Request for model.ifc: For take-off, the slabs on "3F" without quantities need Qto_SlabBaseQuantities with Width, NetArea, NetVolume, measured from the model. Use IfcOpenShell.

First a look at what the model holds.

```python
import ifcopenshell
import ifcopenshell.util.element
import ifcopenshell.util.unit

model = ifcopenshell.open("model.ifc")
print(model.schema)
for unit_type in ("LENGTHUNIT", "AREAUNIT", "VOLUMEUNIT"):
    print(unit_type, ifcopenshell.util.unit.calculate_unit_scale(model, unit_type))
storey = next(s for s in model.by_type("IfcBuildingStorey") if s.Name == "3F")
slabs = [e for e in ifcopenshell.util.element.get_decomposition(storey) if e.is_a("IfcSlab")]
for e in sorted(slabs, key=lambda e: e.id()):
    print(e.id(), e.is_a(), e.Name, list(ifcopenshell.util.element.get_psets(e, qtos_only=True)), sep=" | ")
```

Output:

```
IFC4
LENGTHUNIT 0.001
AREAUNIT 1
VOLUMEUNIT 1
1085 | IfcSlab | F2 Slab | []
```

```python
import ifcopenshell
import ifcopenshell.api.pset
import ifcopenshell.geom
import ifcopenshell.util.element
import ifcopenshell.util.shape
import ifcopenshell.util.unit

model = ifcopenshell.open("model.ifc")
unit_scale = ifcopenshell.util.unit.calculate_unit_scale(model)
area_scale = ifcopenshell.util.unit.calculate_unit_scale(model, "AREAUNIT")
volume_scale = ifcopenshell.util.unit.calculate_unit_scale(model, "VOLUMEUNIT")
settings = ifcopenshell.geom.settings()

storey = next(s for s in model.by_type("IfcBuildingStorey") if s.Name == "3F")
slabs = [e for e in ifcopenshell.util.element.get_decomposition(storey) if e.is_a("IfcSlab")]

for e in sorted(slabs, key=lambda e: e.id()):
    if ifcopenshell.util.element.get_psets(e, qtos_only=True, should_inherit=False):
        continue
    # Geometry comes back in metres, in the element's own axes.
    shape = ifcopenshell.geom.create_shape(settings, e)
    values = {
        "Width": ifcopenshell.util.shape.get_z(shape.geometry) / unit_scale,
        "NetArea": ifcopenshell.util.shape.get_footprint_area(shape.geometry) / area_scale,
        "NetVolume": ifcopenshell.util.shape.get_volume(shape.geometry) / volume_scale,
    }
    qto = ifcopenshell.api.pset.add_qto(model, product=e, name="Qto_SlabBaseQuantities")
    ifcopenshell.api.pset.edit_qto(model, qto=qto, properties=values)
    print(e.id(), {k: round(v, 3) for k, v in values.items()})

model.write("model_rev.ifc")
```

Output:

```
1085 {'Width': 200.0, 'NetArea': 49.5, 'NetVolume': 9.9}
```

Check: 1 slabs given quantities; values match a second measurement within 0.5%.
